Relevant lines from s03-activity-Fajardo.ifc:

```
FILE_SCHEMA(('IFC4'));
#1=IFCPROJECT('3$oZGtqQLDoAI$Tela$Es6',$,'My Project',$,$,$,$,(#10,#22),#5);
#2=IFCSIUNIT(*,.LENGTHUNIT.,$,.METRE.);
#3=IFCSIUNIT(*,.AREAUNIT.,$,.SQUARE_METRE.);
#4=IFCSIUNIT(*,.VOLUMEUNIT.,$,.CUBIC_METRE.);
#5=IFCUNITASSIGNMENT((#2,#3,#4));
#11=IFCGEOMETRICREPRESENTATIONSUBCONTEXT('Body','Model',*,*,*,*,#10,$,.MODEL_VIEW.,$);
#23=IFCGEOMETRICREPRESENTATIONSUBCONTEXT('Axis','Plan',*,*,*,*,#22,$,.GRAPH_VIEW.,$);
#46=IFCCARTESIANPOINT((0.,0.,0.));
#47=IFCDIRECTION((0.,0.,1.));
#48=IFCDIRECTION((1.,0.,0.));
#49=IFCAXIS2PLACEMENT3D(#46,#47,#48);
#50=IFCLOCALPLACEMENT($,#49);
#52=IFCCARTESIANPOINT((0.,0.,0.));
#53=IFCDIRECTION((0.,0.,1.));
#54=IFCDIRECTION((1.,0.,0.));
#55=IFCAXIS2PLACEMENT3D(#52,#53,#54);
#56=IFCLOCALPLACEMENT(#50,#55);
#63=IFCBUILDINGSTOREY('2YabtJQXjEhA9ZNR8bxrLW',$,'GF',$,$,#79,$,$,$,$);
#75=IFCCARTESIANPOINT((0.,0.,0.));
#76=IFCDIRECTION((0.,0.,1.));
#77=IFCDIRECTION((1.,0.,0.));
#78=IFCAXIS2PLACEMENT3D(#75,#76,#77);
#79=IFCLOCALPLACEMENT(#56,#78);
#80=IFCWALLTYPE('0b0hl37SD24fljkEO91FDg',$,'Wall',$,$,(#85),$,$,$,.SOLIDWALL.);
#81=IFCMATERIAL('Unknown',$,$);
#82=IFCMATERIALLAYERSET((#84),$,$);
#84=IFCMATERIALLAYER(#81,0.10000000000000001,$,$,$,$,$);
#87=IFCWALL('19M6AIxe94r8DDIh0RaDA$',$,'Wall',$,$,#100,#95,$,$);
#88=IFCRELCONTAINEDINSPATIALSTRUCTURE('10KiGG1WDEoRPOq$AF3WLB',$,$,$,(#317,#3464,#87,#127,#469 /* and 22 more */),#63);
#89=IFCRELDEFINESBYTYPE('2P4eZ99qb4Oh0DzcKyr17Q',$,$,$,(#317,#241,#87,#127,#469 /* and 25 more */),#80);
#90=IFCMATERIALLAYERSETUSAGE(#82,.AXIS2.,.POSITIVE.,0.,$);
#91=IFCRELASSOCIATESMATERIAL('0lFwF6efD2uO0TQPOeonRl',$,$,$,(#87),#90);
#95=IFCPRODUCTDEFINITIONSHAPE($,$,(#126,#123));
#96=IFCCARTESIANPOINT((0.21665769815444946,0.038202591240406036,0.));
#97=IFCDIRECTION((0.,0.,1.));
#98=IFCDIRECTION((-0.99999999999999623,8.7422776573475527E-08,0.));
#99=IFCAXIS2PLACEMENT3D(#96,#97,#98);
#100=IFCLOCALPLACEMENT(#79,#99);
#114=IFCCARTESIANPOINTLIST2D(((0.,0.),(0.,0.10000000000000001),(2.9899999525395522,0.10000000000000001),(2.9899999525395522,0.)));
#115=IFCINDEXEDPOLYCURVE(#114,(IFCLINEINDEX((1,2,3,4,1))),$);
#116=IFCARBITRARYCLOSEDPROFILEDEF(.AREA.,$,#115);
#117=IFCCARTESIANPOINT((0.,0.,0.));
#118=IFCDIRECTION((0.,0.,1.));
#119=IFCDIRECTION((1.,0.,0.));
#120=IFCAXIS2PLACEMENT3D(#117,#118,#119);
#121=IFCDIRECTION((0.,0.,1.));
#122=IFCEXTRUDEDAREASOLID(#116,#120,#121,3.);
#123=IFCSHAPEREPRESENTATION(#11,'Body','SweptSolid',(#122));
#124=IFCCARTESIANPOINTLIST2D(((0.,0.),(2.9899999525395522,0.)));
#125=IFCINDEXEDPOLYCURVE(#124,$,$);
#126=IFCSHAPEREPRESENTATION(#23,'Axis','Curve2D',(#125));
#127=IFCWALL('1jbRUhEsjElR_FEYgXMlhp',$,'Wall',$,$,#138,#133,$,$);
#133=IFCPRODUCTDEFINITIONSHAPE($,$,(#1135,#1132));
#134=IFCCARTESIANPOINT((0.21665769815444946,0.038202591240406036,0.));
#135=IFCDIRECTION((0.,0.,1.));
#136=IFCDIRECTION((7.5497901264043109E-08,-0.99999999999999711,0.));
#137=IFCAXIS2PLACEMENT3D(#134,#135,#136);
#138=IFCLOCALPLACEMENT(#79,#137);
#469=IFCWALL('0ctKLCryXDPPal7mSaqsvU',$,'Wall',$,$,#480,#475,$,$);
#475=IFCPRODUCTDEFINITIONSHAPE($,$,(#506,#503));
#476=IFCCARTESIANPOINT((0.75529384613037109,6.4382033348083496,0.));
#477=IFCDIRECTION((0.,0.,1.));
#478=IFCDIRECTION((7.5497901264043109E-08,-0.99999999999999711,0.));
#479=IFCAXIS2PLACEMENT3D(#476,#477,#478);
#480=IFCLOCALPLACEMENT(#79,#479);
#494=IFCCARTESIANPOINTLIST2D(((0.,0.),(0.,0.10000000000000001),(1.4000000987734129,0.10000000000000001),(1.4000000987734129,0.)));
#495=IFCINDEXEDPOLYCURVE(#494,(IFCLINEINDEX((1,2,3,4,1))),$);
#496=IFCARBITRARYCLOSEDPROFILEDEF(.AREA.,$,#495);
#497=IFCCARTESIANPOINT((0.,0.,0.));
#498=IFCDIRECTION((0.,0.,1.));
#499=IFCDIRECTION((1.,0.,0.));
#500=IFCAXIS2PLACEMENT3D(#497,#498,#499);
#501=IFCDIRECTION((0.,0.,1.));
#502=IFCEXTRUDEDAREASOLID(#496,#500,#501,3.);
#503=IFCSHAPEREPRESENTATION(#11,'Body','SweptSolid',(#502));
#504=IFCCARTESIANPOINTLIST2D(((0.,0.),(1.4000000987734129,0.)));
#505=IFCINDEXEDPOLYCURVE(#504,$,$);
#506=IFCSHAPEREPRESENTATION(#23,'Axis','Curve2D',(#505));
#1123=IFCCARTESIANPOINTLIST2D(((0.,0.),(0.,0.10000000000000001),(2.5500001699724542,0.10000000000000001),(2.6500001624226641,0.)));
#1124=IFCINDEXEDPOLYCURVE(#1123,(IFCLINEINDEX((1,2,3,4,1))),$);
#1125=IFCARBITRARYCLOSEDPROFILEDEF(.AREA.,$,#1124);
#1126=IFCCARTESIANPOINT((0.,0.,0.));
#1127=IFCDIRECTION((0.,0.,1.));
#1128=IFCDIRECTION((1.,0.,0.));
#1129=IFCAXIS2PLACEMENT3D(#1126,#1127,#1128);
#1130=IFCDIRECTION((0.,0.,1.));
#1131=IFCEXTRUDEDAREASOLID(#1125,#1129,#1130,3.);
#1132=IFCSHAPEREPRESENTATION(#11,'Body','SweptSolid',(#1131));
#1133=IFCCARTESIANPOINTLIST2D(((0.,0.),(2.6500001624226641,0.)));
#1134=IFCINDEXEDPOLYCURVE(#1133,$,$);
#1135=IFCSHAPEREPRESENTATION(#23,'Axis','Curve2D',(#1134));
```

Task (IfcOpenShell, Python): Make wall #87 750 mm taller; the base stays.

```python
import ifcopenshell
import ifcopenshell.geom
import ifcopenshell.util.representation
import ifcopenshell.util.shape

model = ifcopenshell.open("s03-activity-Fajardo.ifc")
settings = ifcopenshell.geom.settings()


def volume(element):
    """Net volume in cubic metres, openings subtracted."""
    shape = ifcopenshell.geom.create_shape(settings, element)
    return ifcopenshell.util.shape.get_volume(shape.geometry)


wall = model.by_guid("19M6AIxe94r8DDIh0RaDA$")
before = volume(wall)

body = ifcopenshell.util.representation.get_representation(wall, "Model", "Body")
solid = body.Items[0]
old_height = solid.Depth
solid.Depth += 0.75
after = volume(wall)

print(f"height {old_height:g} -> {solid.Depth:g}, volume {before:.3f} -> {after:.3f} m3")

model.write("s03-activity-Fajardo-out.ifc")
```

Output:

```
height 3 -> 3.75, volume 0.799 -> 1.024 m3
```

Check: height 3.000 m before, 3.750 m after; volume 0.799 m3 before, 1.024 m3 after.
